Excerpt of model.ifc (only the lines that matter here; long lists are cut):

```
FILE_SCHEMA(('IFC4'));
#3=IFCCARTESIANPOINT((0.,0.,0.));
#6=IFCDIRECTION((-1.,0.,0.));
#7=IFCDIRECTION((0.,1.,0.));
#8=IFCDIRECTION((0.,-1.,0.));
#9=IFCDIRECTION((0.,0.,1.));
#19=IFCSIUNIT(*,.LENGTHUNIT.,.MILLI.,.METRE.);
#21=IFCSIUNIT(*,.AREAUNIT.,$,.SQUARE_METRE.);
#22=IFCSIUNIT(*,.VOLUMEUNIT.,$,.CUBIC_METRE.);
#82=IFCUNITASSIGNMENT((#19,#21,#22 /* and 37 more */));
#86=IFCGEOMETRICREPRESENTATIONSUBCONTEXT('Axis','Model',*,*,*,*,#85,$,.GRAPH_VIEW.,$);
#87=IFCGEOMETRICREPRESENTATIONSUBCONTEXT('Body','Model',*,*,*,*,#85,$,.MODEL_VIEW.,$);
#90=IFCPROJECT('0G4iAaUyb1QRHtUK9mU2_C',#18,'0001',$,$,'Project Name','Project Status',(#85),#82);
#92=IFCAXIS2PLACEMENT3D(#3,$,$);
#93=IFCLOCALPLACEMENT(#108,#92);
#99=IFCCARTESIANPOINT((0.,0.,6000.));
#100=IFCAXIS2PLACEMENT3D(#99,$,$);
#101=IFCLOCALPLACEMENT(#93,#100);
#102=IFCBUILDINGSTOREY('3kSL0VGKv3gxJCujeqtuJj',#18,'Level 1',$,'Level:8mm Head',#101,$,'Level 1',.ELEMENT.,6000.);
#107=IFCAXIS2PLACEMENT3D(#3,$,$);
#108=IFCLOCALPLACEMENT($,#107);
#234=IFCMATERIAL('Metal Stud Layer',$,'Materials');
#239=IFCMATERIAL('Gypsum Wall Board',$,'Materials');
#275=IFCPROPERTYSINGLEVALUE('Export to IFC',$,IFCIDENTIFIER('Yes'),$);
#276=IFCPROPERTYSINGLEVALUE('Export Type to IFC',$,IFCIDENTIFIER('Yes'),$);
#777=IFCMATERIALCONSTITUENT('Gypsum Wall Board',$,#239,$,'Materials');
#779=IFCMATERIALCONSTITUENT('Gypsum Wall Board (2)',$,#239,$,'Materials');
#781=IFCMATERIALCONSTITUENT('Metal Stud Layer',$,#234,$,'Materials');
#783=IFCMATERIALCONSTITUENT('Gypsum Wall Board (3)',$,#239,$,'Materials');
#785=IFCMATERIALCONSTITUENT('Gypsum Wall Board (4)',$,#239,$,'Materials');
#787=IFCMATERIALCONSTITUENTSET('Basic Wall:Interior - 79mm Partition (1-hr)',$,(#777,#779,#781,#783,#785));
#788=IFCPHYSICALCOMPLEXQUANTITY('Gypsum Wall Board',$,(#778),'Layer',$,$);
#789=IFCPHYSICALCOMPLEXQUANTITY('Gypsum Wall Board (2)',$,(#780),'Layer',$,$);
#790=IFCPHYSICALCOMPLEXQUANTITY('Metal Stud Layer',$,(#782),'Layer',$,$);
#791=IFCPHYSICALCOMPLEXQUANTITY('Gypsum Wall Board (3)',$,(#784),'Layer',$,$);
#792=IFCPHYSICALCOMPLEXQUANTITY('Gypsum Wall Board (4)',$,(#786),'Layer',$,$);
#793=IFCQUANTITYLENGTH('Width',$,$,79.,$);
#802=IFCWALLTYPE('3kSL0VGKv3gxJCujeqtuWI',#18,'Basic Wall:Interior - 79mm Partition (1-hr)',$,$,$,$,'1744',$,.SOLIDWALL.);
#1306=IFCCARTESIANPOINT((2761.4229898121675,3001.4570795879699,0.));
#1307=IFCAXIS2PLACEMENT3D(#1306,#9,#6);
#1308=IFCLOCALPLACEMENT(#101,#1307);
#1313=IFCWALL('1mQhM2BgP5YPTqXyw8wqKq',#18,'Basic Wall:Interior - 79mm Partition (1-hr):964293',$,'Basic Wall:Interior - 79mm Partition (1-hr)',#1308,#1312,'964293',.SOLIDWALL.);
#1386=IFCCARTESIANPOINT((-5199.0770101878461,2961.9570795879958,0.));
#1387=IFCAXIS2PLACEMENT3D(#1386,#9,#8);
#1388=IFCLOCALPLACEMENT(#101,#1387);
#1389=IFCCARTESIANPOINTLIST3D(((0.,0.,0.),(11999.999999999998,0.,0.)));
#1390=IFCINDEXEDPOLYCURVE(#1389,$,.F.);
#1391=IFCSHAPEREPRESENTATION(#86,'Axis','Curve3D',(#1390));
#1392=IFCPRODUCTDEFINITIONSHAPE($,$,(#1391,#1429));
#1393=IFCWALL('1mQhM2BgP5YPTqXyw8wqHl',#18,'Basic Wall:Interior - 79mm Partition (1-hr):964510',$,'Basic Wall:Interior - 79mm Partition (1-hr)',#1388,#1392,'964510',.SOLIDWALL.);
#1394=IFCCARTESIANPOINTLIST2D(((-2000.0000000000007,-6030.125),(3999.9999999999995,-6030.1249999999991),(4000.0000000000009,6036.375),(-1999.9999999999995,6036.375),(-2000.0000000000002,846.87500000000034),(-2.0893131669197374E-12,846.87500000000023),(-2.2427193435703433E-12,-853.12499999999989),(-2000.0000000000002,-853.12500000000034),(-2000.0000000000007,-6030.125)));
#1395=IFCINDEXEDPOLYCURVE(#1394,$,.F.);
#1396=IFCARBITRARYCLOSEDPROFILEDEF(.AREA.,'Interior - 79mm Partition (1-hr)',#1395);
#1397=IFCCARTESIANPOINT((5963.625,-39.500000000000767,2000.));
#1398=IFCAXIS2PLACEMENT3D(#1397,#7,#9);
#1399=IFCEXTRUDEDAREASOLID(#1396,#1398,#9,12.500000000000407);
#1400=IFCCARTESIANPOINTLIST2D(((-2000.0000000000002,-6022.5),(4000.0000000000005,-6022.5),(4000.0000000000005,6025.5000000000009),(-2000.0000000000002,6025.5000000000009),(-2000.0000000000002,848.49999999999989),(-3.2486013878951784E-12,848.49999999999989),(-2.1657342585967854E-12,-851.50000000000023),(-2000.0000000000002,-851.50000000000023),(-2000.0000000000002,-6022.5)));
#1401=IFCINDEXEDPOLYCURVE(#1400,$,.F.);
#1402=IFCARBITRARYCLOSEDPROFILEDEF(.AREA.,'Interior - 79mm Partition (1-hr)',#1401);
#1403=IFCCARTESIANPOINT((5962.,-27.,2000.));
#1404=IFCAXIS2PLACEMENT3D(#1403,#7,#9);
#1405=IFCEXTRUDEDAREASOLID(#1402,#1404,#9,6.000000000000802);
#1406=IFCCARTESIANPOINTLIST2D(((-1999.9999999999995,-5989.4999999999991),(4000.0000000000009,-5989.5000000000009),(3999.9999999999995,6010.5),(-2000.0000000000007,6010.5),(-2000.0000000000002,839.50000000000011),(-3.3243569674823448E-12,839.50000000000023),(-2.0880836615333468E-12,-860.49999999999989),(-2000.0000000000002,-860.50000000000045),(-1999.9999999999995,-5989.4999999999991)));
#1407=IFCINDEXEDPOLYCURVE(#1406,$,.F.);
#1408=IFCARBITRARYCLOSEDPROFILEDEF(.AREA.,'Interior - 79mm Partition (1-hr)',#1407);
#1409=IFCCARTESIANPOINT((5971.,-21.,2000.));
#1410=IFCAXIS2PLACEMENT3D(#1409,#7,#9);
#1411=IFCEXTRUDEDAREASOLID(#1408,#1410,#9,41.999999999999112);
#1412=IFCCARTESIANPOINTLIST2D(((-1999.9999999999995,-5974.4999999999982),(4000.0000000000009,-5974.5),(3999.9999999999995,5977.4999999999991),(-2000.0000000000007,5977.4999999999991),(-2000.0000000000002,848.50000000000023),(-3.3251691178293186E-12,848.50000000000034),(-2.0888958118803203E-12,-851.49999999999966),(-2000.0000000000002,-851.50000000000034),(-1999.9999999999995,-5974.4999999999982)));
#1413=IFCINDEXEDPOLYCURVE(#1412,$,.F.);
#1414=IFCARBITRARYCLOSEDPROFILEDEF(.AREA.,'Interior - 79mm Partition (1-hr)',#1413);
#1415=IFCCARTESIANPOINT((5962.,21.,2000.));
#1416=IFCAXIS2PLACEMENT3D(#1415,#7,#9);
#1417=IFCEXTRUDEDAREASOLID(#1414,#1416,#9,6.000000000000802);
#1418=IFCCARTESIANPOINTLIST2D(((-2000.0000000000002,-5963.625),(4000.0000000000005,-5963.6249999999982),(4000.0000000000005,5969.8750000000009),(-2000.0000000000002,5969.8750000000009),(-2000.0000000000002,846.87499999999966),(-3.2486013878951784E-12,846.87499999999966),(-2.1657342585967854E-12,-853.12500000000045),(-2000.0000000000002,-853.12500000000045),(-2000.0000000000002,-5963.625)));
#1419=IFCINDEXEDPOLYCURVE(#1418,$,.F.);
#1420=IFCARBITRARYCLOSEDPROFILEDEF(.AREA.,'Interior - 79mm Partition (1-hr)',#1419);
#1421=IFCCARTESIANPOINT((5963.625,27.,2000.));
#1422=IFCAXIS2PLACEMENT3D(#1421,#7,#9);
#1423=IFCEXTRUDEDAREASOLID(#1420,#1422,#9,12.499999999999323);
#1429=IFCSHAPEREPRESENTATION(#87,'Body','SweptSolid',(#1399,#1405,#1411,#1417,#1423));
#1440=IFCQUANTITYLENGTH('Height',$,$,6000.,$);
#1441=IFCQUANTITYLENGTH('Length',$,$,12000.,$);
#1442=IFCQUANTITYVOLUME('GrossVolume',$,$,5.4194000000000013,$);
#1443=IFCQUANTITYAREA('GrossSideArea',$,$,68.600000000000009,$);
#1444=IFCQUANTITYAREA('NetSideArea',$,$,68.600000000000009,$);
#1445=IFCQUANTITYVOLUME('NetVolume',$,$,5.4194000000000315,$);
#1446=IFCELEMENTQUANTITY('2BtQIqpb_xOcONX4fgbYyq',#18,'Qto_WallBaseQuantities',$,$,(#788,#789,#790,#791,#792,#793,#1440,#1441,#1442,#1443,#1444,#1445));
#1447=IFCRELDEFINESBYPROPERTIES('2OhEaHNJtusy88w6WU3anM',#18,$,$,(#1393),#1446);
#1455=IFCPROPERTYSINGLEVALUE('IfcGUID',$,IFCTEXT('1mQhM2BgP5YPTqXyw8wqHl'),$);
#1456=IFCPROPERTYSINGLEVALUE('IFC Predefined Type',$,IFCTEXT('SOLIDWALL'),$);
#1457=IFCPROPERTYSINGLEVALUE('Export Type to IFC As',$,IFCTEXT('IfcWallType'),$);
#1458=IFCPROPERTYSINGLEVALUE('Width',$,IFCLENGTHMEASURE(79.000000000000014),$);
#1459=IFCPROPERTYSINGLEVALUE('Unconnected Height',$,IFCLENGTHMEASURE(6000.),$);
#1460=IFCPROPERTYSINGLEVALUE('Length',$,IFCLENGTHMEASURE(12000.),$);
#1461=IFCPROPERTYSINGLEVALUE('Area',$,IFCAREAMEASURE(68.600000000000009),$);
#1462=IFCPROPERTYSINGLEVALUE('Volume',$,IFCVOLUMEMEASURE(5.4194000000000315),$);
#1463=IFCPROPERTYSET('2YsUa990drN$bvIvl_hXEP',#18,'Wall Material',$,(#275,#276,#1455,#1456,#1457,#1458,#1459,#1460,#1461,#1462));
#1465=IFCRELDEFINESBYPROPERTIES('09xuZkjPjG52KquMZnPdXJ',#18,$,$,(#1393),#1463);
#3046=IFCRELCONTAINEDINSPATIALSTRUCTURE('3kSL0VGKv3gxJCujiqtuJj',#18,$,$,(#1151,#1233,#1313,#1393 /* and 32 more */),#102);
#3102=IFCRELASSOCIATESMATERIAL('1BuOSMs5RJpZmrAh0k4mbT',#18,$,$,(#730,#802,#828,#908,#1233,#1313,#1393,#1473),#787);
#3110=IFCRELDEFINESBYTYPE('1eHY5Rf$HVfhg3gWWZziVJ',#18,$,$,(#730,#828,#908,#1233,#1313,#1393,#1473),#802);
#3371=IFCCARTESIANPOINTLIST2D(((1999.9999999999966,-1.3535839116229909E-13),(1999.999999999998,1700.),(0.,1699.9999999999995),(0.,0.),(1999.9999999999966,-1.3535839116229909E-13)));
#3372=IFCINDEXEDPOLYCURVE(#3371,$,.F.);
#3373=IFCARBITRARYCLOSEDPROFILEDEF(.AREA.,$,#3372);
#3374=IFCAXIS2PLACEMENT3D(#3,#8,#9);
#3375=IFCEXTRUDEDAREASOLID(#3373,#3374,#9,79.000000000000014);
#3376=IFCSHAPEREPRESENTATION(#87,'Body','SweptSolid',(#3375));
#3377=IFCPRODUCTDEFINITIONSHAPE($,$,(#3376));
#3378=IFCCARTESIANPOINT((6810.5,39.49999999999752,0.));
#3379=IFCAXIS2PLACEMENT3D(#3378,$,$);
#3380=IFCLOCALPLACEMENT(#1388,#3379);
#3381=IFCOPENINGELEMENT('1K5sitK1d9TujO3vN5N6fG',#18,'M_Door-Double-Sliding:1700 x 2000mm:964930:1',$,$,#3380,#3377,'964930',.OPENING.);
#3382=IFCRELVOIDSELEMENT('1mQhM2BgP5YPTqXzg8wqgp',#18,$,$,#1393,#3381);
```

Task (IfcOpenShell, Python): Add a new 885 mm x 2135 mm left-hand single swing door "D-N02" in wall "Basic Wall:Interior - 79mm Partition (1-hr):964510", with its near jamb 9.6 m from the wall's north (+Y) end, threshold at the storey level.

```python
import numpy as np
import ifcopenshell
import ifcopenshell.api.feature
import ifcopenshell.api.geometry
import ifcopenshell.api.pset
import ifcopenshell.api.root
import ifcopenshell.api.spatial
import ifcopenshell.geom
import ifcopenshell.util.element
import ifcopenshell.util.placement
import ifcopenshell.util.representation
import ifcopenshell.util.shape
import ifcopenshell.util.unit

model = ifcopenshell.open("model.ifc")
unit_scale = ifcopenshell.util.unit.calculate_unit_scale(model)
area_scale = ifcopenshell.util.unit.calculate_unit_scale(model, "AREAUNIT")
volume_scale = ifcopenshell.util.unit.calculate_unit_scale(model, "VOLUMEUNIT")
settings = ifcopenshell.geom.settings()


def volume(element):
    """Net volume in cubic metres, openings subtracted."""
    shape = ifcopenshell.geom.create_shape(settings, element)
    return ifcopenshell.util.shape.get_volume(shape.geometry)


wall = model.by_guid("1mQhM2BgP5YPTqXyw8wqHl")
storey = ifcopenshell.util.element.get_container(wall, ifc_class="IfcBuildingStorey")
context = ifcopenshell.util.representation.get_context(model, "Model", "Body", "MODEL_VIEW")
before = volume(wall)

width, height, from_end, sill = 0.885, 2.135, 9.6, 0.0  # metres

# The wall runs along its own X axis, and the end named is its -X end.
wall_shape = ifcopenshell.geom.create_shape(settings, wall)
x, y, z = ifcopenshell.util.shape.get_vertices(wall_shape.geometry).T
start = x.min() + from_end
face, thickness = float(y.min()), float(y.max() - y.min())
wall_matrix = ifcopenshell.util.placement.get_local_placement(wall.ObjectPlacement)
level = ifcopenshell.util.placement.get_local_placement(storey.ObjectPlacement)[2, 3]


def in_wall(x, y):
    """Placement at x, y metres in the wall's axes, at sill height."""
    matrix = wall_matrix.copy()
    matrix[:, 3] = wall_matrix @ np.array([x / unit_scale, y / unit_scale, 0.0, 1.0])
    matrix[2, 3] = level + sill / unit_scale
    return matrix


# Opening: a box that overshoots both wall faces by 50 mm.
opening = ifcopenshell.api.root.create_entity(model, ifc_class="IfcOpeningElement", predefined_type="OPENING")
box = ifcopenshell.api.geometry.add_wall_representation(
    model, context=context, length=width, height=height, thickness=thickness + 0.1
)
ifcopenshell.api.geometry.assign_representation(model, product=opening, representation=box)
ifcopenshell.api.geometry.edit_object_placement(model, product=opening, matrix=in_wall(start, face - 0.05), is_si=False)
ifcopenshell.api.feature.add_feature(model, feature=opening, element=wall)

door = ifcopenshell.api.root.create_entity(model, ifc_class="IfcDoor", name="D-N02", predefined_type="DOOR")
door.OverallWidth, door.OverallHeight = width / unit_scale, height / unit_scale
door.OperationType = "SINGLE_SWING_LEFT"
body = ifcopenshell.api.geometry.add_door_representation(
    model,
    context=context,
    overall_width=door.OverallWidth,
    overall_height=door.OverallHeight,
    operation_type="SINGLE_SWING_LEFT",
    lining_properties={"LiningDepth": thickness / unit_scale, "ThresholdDepth": thickness / unit_scale},
)
ifcopenshell.api.geometry.assign_representation(model, product=door, representation=body)
ifcopenshell.api.spatial.assign_container(model, products=[door], relating_structure=storey)
ifcopenshell.api.feature.add_filling(model, opening=opening, element=door)

# The lining spans the wall, so the door starts at the wall face.
ifcopenshell.api.geometry.edit_object_placement(model, product=door, matrix=in_wall(start, face), is_si=False)

after = volume(wall)

# Update the wall's stored quantities.
qto = model.by_id(ifcopenshell.util.element.get_pset(wall, "Qto_WallBaseQuantities", should_inherit=False)["id"])
ifcopenshell.api.pset.edit_qto(model, qto=qto, properties={
    "NetSideArea": after / thickness / area_scale,
    "NetVolume": after / volume_scale,
})
pset = model.by_id(ifcopenshell.util.element.get_pset(wall, "Wall Material", should_inherit=False)["id"])
ifcopenshell.api.pset.edit_pset(model, pset=pset, properties={
    "Area": model.create_entity("IfcAreaMeasure", after / thickness / area_scale),
    "Volume": model.create_entity("IfcVolumeMeasure", after / volume_scale),
})

print(f"wall volume {before:.3f} -> {after:.3f} m3")

model.write("model_v2.ifc")
```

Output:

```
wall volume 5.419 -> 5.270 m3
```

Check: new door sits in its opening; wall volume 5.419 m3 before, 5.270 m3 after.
